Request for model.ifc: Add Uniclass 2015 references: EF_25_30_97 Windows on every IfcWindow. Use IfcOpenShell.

First a look at what the model holds.

```python
import ifcopenshell

model = ifcopenshell.open("model.ifc")
print(model.schema)
print("classifications:", [c.Name for c in model.by_type("IfcClassification")])
for ifc_class in ("IfcDoor", "IfcRoof", "IfcStair", "IfcWall", "IfcWindow"):
    print(ifc_class, len(model.by_type(ifc_class)))
```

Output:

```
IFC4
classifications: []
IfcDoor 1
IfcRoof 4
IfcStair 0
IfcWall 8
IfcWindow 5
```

```python
import ifcopenshell
import ifcopenshell.api.classification

model = ifcopenshell.open("model.ifc")

system = ifcopenshell.api.classification.add_classification(model, classification="Uniclass 2015")

codes = {
    "IfcWindow": ("EF_25_30_97", "Windows"),
}
for ifc_class, (code, name) in codes.items():
    products = model.by_type(ifc_class)
    ifcopenshell.api.classification.add_reference(
        model, products=products, classification=system, identification=code, name=name
    )
    print(code, len(products))

model.write("model-out.ifc")
```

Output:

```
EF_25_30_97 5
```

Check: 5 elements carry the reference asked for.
